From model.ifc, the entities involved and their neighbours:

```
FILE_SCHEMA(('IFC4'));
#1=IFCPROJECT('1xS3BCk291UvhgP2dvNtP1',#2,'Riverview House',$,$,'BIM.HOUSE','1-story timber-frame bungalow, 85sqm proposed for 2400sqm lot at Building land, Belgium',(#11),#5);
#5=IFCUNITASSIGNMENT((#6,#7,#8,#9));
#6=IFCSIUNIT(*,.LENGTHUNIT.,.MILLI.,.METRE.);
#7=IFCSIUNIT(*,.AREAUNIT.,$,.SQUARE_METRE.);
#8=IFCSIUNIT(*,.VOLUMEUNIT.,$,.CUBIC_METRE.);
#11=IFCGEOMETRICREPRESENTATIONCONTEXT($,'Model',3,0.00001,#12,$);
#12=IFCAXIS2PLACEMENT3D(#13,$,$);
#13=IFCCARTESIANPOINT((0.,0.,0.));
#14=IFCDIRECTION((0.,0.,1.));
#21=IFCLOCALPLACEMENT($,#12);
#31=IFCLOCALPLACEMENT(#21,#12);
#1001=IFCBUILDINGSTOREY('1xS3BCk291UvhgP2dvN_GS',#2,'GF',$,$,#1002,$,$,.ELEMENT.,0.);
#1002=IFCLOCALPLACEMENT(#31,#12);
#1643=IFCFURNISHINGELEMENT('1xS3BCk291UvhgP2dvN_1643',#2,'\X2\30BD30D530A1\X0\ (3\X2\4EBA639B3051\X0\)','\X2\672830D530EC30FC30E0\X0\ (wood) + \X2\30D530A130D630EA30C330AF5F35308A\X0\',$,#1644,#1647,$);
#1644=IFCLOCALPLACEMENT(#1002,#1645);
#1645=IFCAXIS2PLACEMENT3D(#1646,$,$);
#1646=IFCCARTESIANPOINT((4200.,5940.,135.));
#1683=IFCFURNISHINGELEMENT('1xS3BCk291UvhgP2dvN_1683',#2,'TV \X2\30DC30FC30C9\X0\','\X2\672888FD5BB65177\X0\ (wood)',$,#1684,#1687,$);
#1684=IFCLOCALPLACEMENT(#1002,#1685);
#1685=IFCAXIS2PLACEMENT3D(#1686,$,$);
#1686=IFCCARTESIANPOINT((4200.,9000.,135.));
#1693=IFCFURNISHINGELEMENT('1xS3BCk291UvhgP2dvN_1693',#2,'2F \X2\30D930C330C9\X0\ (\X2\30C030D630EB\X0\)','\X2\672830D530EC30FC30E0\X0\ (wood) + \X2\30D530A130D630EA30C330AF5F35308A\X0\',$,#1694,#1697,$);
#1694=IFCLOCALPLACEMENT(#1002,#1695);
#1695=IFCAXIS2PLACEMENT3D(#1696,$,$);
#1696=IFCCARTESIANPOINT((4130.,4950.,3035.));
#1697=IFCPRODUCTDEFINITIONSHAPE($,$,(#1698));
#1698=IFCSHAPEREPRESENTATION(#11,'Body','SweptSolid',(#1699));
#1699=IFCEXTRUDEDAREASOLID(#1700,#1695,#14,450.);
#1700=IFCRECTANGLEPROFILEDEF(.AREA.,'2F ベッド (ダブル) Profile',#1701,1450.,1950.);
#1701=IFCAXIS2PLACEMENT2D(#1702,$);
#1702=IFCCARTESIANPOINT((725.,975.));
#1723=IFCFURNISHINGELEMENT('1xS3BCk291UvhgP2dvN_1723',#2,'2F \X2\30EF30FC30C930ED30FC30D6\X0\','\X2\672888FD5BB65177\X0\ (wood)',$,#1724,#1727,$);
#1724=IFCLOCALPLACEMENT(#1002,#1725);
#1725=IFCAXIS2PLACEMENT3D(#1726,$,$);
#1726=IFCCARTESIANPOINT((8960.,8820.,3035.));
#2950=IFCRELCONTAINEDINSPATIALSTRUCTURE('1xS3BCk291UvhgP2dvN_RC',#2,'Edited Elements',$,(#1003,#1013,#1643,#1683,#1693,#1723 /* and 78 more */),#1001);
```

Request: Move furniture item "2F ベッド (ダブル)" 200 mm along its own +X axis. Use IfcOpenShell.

```python
import ifcopenshell
import ifcopenshell.api.geometry
import ifcopenshell.util.placement
import ifcopenshell.util.unit

model = ifcopenshell.open("model.ifc")
unit_scale = ifcopenshell.util.unit.calculate_unit_scale(model)

item = model.by_guid("1xS3BCk291UvhgP2dvN_1693")
matrix = ifcopenshell.util.placement.get_local_placement(item.ObjectPlacement)
matrix[:3, 3] += matrix[:3, 0] * 0.2 / unit_scale
ifcopenshell.api.geometry.edit_object_placement(model, product=item, matrix=matrix, is_si=False)

print(ifcopenshell.util.placement.get_local_placement(item.ObjectPlacement).round(3) + 0.0)

model.write("model_edited.ifc")
```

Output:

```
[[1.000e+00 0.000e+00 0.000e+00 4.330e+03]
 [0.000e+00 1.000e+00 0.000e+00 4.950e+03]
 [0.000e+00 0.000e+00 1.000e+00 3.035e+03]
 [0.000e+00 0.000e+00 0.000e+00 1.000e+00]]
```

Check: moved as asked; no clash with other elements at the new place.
